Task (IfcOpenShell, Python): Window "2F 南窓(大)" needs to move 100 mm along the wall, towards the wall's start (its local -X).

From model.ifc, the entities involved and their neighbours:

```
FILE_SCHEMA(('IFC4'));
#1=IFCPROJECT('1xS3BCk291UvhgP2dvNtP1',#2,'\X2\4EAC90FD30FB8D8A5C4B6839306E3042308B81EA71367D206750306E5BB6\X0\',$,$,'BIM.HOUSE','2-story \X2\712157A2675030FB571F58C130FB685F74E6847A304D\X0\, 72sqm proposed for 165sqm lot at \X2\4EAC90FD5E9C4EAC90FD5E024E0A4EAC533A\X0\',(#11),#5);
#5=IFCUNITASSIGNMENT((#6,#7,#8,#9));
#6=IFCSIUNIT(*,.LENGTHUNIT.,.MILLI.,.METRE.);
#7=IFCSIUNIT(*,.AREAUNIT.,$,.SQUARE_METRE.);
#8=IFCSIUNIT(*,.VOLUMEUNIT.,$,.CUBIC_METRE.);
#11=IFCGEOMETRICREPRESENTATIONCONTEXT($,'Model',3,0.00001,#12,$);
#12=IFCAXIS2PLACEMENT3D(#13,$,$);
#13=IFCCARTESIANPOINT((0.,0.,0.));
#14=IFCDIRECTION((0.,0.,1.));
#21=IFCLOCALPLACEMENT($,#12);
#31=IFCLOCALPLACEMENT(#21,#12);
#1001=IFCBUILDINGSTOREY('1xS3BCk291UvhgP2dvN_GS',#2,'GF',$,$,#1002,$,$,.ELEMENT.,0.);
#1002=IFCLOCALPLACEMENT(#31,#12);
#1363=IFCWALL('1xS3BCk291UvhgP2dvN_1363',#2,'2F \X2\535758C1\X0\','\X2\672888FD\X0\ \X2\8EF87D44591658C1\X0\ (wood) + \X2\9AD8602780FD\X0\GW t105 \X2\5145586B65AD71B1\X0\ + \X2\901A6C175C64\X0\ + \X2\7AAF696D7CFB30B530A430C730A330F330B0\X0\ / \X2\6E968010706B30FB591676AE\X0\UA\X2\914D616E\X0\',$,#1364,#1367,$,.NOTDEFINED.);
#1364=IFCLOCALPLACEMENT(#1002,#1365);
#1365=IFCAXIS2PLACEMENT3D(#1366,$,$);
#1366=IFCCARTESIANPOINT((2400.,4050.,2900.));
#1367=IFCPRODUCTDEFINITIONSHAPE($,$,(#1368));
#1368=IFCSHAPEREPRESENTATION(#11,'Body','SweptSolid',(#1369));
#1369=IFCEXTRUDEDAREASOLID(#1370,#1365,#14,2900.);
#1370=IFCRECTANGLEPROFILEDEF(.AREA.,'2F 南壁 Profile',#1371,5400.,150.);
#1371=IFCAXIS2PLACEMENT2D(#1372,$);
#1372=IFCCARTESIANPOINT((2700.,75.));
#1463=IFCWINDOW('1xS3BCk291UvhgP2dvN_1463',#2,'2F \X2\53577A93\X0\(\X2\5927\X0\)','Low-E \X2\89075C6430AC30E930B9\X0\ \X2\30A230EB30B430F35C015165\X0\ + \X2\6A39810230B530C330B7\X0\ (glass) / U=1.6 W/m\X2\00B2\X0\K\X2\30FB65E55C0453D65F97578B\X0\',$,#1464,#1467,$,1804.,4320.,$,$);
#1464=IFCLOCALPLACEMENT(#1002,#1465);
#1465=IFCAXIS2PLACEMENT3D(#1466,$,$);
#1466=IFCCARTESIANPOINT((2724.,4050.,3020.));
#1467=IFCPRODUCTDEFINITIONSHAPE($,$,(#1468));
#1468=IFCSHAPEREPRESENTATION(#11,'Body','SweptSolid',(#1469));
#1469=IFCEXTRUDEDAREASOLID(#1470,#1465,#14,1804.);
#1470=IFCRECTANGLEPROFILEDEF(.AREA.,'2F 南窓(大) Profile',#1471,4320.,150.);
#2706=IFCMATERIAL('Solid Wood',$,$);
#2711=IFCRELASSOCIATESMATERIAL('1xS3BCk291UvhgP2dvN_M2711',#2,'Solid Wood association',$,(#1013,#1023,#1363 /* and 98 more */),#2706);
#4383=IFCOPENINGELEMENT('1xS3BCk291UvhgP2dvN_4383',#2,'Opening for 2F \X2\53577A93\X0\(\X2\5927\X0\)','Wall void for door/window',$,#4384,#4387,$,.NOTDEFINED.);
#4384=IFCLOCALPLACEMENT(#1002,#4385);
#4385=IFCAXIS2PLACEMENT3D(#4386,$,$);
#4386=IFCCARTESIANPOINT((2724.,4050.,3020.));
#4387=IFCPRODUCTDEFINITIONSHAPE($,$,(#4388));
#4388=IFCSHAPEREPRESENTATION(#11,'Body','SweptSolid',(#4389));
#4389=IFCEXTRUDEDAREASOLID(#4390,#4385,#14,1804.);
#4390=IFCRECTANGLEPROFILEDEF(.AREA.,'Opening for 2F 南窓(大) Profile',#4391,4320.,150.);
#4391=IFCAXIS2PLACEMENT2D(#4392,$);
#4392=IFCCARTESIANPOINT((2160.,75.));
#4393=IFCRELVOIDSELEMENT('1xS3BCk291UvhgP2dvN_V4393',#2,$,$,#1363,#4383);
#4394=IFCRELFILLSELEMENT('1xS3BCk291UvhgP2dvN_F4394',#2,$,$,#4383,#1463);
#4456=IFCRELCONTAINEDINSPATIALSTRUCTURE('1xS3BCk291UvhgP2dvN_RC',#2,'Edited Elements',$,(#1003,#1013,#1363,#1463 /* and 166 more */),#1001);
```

```python
import ifcopenshell
import ifcopenshell.api.geometry
import ifcopenshell.util.placement

model = ifcopenshell.open("model.ifc")

window = model.by_guid("1xS3BCk291UvhgP2dvN_1463")
opening = window.FillsVoids[0].RelatingOpeningElement
wall = opening.VoidsElements[0].RelatingBuildingElement

wall_matrix = ifcopenshell.util.placement.get_local_placement(wall.ObjectPlacement)
shift = wall_matrix[:3, 0] * -100.0
before = ifcopenshell.util.placement.get_local_placement(window.ObjectPlacement)[:3, 3].copy()

# The window is not placed relative to its opening, so move both.
for product in (opening, window):
    matrix = ifcopenshell.util.placement.get_local_placement(product.ObjectPlacement)
    matrix[:3, 3] += shift
    ifcopenshell.api.geometry.edit_object_placement(model, product=product, matrix=matrix, is_si=False)

after = ifcopenshell.util.placement.get_local_placement(window.ObjectPlacement)[:3, 3]
print("window moved by", (after - before).round(3) + 0.0)

model.write("model-out.ifc")
```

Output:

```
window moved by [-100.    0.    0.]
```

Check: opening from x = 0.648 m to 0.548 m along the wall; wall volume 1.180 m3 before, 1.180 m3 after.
